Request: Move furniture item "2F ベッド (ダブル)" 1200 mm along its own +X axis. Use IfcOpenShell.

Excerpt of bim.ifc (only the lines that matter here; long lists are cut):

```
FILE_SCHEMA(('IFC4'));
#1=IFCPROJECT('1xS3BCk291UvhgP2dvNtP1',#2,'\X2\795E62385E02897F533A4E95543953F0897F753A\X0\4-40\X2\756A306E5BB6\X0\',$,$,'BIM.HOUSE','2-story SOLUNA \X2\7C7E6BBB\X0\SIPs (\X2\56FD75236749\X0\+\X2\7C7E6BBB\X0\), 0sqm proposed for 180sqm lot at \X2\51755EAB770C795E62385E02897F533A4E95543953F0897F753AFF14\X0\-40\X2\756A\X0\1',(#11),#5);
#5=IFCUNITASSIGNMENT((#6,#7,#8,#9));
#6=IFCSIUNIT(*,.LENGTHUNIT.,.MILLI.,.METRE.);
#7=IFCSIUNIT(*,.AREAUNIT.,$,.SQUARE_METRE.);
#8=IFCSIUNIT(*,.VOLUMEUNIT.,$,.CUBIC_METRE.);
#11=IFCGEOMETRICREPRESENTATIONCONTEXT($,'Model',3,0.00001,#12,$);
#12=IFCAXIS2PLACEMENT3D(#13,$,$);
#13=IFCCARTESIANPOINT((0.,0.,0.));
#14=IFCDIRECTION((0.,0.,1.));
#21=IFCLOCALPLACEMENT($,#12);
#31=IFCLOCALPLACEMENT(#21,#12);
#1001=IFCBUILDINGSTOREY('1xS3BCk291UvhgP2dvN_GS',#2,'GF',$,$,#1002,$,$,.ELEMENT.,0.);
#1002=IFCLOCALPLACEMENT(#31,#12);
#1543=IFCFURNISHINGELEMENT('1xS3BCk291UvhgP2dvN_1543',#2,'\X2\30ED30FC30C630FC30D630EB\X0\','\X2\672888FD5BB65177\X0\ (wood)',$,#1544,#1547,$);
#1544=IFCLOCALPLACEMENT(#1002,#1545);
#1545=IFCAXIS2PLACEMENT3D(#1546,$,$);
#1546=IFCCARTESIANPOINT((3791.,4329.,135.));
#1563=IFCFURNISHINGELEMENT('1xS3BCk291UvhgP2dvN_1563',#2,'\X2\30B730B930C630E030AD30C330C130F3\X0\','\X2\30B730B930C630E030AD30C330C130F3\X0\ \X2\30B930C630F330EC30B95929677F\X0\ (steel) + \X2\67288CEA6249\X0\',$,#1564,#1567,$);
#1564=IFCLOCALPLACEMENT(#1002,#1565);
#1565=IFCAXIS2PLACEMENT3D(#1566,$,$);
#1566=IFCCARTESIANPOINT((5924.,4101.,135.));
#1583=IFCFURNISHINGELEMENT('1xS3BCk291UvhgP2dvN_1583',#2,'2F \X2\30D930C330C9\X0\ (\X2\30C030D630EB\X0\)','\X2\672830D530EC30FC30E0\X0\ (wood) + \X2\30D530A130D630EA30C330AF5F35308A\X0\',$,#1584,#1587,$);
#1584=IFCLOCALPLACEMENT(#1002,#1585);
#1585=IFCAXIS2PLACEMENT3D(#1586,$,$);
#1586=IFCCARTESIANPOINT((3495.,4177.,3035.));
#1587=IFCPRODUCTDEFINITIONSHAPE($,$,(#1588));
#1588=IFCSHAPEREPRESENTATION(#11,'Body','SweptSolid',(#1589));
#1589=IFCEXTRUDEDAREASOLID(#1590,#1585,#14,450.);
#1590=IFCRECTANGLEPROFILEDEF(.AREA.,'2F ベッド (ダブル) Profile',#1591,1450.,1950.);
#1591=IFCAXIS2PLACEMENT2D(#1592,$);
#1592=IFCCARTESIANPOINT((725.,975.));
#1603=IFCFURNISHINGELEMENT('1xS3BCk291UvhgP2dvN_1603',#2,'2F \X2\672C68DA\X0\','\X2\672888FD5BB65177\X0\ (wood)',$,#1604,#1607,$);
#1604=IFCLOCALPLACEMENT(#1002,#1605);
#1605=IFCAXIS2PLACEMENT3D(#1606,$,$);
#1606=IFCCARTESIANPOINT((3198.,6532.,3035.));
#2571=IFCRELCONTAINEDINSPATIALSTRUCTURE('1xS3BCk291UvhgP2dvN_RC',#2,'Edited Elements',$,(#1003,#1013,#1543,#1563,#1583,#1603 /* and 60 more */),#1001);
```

```python
import ifcopenshell
import ifcopenshell.api.geometry
import ifcopenshell.util.placement
import ifcopenshell.util.unit

model = ifcopenshell.open("bim.ifc")
unit_scale = ifcopenshell.util.unit.calculate_unit_scale(model)

item = model.by_id(1583)
matrix = ifcopenshell.util.placement.get_local_placement(item.ObjectPlacement)
matrix[:3, 3] += matrix[:3, 0] * 1.2 / unit_scale
ifcopenshell.api.geometry.edit_object_placement(model, product=item, matrix=matrix, is_si=False)

print(ifcopenshell.util.placement.get_local_placement(item.ObjectPlacement).round(3) + 0.0)

model.write("bim-out.ifc")
```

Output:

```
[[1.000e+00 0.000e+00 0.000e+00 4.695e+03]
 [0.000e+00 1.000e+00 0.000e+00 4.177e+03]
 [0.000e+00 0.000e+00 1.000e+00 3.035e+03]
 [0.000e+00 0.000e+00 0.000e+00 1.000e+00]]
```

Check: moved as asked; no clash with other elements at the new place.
